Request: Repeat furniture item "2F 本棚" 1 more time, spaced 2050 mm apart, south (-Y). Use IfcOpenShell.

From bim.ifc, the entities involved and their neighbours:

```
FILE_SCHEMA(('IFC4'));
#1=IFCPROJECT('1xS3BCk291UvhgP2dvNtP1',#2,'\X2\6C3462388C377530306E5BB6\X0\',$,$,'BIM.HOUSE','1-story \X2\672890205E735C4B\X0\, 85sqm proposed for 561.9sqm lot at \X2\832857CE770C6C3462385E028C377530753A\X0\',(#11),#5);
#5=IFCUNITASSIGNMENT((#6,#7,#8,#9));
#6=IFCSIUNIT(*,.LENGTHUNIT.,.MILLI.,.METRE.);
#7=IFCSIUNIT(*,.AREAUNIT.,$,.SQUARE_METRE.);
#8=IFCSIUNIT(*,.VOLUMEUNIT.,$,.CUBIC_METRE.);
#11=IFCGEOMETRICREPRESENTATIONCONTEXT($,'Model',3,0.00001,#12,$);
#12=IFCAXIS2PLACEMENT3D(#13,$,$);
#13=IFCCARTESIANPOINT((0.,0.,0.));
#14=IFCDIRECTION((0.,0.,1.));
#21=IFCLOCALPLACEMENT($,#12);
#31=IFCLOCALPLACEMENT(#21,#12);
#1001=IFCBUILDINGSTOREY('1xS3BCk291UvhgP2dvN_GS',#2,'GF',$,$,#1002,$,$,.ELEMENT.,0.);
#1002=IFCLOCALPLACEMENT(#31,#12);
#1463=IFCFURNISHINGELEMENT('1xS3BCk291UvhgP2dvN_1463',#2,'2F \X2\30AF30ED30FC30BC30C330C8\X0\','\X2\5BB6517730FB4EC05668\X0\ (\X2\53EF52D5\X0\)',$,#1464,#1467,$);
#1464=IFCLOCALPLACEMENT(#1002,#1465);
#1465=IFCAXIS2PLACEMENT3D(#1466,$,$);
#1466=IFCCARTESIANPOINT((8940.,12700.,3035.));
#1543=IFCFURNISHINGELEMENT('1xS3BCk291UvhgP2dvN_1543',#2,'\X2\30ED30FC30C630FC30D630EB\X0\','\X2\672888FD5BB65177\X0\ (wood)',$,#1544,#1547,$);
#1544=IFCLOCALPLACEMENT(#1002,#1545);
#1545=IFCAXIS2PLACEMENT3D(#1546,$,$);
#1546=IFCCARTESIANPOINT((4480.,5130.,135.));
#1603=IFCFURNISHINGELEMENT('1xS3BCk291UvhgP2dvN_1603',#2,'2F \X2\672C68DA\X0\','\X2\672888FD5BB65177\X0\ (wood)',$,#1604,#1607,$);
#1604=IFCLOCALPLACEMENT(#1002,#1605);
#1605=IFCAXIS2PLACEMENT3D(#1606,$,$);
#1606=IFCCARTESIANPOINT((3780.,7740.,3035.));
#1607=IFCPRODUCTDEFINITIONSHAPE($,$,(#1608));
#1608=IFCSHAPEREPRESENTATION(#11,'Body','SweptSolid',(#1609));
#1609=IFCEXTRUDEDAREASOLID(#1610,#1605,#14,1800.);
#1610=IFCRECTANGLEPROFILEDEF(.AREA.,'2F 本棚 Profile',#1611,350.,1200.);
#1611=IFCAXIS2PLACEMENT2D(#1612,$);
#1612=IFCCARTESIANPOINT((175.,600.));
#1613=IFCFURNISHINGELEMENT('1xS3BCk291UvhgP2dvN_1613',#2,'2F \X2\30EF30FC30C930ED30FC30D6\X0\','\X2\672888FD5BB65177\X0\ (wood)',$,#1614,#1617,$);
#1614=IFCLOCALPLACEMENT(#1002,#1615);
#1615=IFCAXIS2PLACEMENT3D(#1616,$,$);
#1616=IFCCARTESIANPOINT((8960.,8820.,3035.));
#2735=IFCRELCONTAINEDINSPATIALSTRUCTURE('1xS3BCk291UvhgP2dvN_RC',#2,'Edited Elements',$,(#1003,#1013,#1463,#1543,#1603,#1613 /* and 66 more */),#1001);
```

```python
import numpy as np
import ifcopenshell
import ifcopenshell.api.geometry
import ifcopenshell.api.root
import ifcopenshell.util.element
import ifcopenshell.util.placement
import ifcopenshell.util.unit

model = ifcopenshell.open("bim.ifc")
unit_scale = ifcopenshell.util.unit.calculate_unit_scale(model)


def reuse_history(source, copy):
    """copy_class also copies each property set's owner history, people and application; keep the originals."""
    for rel in copy.IsDefinedBy:
        if rel.is_a("IfcRelDefinesByProperties") and (history := rel.RelatingPropertyDefinition.OwnerHistory):
            rel.RelatingPropertyDefinition.OwnerHistory = source.OwnerHistory
            ifcopenshell.util.element.remove_deep2(model, history)


source = model.by_id(1603)
base = ifcopenshell.util.placement.get_local_placement(source.ObjectPlacement)
step = np.array([0.0, -1.0, 0.0]) * 2.05 / unit_scale

for i in range(1, 2):
    copy = ifcopenshell.api.root.copy_class(model, product=source)
    copy.Representation = ifcopenshell.util.element.copy_deep(
        model, source.Representation, exclude=["IfcGeometricRepresentationContext", "IfcRepresentationMap"]
    )
    reuse_history(source, copy)
    matrix = base.copy()
    matrix[:3, 3] += i * step
    print("added at", matrix[:3, 3].round(3) + 0.0)
    ifcopenshell.api.geometry.edit_object_placement(model, product=copy, matrix=matrix, is_si=False)

model.write("bim_updated.ifc")
```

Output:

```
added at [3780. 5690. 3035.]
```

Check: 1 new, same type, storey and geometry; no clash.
